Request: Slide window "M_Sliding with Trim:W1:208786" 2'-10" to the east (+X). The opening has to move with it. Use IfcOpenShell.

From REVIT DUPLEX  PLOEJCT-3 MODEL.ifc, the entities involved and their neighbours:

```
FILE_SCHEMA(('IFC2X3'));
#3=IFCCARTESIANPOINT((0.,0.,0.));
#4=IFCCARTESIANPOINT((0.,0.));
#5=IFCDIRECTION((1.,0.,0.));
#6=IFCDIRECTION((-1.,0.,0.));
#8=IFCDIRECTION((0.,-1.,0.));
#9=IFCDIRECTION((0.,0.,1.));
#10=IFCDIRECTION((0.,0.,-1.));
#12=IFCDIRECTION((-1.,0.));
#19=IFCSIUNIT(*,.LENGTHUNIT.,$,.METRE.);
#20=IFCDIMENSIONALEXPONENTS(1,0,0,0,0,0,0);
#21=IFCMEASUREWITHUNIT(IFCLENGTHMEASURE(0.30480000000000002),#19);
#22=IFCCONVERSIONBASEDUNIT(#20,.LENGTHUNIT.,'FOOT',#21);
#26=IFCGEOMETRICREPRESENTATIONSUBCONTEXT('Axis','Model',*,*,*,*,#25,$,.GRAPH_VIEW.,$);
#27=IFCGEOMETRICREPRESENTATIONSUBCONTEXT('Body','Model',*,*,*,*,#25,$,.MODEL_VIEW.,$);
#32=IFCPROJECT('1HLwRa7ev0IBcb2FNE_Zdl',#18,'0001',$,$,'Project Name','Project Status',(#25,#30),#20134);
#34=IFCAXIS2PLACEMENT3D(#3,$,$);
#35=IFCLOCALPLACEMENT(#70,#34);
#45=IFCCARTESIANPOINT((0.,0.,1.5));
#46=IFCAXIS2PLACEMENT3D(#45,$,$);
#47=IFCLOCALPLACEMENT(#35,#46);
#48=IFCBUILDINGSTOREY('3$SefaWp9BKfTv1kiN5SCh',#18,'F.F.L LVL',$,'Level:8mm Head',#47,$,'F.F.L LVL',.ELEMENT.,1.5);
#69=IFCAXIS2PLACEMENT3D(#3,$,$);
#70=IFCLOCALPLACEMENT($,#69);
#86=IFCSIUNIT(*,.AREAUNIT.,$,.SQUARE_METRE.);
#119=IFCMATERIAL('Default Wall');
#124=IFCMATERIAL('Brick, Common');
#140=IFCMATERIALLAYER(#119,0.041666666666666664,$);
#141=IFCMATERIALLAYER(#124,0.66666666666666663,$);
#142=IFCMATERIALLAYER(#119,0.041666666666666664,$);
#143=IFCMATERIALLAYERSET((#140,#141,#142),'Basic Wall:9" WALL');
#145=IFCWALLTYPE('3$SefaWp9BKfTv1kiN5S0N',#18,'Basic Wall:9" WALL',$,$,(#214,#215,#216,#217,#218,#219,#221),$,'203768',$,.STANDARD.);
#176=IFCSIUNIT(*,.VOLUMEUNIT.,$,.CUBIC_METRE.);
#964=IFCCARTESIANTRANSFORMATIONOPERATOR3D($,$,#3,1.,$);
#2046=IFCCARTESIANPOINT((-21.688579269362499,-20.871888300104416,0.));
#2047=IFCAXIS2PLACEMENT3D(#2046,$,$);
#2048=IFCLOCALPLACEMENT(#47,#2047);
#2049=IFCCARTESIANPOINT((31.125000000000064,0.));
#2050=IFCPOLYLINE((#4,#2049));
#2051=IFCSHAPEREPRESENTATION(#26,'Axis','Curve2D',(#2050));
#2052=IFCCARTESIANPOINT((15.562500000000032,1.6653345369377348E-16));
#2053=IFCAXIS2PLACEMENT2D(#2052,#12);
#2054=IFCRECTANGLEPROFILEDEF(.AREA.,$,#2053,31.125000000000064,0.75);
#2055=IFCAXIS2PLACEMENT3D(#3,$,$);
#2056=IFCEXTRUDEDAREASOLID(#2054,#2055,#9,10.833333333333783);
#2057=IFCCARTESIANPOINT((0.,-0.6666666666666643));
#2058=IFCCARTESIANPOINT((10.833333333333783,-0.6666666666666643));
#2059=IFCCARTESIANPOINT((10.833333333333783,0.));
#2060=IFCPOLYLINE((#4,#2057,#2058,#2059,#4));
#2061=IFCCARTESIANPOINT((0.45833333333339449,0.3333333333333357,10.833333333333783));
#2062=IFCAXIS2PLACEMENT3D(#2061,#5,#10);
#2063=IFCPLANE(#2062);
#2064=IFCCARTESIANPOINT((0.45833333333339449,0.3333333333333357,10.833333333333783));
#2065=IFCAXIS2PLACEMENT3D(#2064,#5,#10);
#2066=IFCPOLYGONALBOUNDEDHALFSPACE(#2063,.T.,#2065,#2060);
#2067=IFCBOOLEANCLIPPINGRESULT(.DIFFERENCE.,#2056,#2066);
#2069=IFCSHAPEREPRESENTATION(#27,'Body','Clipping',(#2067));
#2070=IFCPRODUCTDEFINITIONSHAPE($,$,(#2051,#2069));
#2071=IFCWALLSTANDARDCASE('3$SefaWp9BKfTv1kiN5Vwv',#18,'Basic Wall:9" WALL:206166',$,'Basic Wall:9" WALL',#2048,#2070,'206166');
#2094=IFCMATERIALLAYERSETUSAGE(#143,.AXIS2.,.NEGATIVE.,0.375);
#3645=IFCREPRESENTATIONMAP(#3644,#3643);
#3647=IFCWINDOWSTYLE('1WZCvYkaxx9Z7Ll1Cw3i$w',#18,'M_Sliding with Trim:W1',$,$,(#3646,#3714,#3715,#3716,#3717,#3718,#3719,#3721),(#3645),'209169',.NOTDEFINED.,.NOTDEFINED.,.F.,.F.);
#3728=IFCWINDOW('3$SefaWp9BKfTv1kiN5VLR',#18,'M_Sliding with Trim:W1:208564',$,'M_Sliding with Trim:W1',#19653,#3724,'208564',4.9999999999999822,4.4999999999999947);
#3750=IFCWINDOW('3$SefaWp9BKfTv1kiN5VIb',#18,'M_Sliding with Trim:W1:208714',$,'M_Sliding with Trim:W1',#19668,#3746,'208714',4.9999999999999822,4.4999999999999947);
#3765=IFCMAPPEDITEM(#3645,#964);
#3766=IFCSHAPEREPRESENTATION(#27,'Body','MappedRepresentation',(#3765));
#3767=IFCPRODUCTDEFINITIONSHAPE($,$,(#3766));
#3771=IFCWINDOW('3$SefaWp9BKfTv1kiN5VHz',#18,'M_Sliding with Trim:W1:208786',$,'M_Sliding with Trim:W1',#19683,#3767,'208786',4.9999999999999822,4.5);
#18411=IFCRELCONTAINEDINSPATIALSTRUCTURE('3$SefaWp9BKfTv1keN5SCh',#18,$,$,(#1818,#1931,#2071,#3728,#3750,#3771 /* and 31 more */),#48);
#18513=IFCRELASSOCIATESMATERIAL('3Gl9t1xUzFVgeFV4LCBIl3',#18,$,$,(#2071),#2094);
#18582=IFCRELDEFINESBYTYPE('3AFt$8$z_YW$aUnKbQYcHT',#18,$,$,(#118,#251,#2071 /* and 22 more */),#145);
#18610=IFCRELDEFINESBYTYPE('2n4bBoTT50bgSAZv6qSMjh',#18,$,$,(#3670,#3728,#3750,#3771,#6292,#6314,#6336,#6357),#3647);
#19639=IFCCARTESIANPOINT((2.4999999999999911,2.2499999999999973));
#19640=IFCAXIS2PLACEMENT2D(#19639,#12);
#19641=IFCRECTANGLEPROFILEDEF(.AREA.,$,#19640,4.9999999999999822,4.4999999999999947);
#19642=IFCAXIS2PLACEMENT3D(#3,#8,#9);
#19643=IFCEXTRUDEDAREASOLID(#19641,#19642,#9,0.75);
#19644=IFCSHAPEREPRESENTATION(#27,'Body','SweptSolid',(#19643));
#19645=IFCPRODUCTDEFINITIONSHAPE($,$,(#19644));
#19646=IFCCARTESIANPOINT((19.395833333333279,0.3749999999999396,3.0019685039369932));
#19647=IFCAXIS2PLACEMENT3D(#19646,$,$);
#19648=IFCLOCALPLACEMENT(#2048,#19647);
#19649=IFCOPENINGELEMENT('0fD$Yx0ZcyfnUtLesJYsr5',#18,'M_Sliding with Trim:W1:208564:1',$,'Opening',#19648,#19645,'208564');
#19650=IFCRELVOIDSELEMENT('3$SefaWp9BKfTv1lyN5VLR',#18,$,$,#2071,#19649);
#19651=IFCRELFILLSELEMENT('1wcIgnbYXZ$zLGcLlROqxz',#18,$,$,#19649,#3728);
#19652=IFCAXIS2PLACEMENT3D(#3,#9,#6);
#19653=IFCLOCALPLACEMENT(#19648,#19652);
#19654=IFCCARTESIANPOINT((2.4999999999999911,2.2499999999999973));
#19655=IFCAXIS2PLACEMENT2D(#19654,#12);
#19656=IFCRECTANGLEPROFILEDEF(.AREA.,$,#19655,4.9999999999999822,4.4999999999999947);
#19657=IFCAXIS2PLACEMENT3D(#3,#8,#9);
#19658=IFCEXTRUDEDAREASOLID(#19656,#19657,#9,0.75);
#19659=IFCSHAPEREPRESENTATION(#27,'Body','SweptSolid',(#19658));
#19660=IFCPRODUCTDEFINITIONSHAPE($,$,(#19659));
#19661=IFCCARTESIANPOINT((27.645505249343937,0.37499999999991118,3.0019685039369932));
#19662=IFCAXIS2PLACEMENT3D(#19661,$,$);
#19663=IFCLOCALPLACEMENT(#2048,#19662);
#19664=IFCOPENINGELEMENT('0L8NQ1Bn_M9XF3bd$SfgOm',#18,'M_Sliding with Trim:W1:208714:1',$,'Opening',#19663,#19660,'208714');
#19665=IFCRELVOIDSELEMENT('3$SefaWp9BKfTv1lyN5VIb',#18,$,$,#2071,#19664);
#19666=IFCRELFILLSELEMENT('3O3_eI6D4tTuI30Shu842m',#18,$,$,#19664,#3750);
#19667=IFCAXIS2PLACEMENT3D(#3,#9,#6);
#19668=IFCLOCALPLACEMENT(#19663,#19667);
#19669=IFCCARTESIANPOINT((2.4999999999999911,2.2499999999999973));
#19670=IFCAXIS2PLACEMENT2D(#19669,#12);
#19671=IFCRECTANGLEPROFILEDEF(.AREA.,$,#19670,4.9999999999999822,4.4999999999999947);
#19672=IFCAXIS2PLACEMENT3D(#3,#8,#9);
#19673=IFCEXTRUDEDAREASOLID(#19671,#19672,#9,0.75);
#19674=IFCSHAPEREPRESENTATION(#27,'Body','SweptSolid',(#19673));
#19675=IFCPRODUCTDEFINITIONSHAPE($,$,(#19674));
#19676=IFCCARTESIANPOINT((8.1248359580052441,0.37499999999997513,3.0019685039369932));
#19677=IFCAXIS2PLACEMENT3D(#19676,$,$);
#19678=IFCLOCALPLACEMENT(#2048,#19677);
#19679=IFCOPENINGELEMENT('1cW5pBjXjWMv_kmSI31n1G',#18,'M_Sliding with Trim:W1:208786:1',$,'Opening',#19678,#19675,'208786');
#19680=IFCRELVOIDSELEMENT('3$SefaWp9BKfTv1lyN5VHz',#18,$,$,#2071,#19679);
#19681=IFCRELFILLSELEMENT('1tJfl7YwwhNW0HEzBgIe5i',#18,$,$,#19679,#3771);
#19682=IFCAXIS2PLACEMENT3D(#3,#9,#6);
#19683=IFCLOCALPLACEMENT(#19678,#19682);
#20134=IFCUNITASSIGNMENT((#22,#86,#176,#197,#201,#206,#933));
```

```python
import ifcopenshell
import ifcopenshell.api.geometry
import ifcopenshell.util.placement
import ifcopenshell.util.unit

model = ifcopenshell.open("REVIT DUPLEX  PLOEJCT-3 MODEL.ifc")
unit_scale = ifcopenshell.util.unit.calculate_unit_scale(model)

window = model.by_guid("3$SefaWp9BKfTv1kiN5VHz")
opening = window.FillsVoids[0].RelatingOpeningElement
wall = opening.VoidsElements[0].RelatingBuildingElement

wall_matrix = ifcopenshell.util.placement.get_local_placement(wall.ObjectPlacement)
shift = wall_matrix[:3, 0] * 34 * 0.0254 / unit_scale
before = ifcopenshell.util.placement.get_local_placement(window.ObjectPlacement)[:3, 3].copy()

# The window is placed relative to its opening, so it follows when the opening moves.
matrix = ifcopenshell.util.placement.get_local_placement(opening.ObjectPlacement)
matrix[:3, 3] += shift
ifcopenshell.api.geometry.edit_object_placement(
    model, product=opening, matrix=matrix, is_si=False, should_transform_children=True
)

after = ifcopenshell.util.placement.get_local_placement(window.ObjectPlacement)[:3, 3]
print("window moved by", (after - before).round(3) + 0.0)

model.write("REVIT DUPLEX  PLOEJCT-3 MODEL_edited.ifc")
```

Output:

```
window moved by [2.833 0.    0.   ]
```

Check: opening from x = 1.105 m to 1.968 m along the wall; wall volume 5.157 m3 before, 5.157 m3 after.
